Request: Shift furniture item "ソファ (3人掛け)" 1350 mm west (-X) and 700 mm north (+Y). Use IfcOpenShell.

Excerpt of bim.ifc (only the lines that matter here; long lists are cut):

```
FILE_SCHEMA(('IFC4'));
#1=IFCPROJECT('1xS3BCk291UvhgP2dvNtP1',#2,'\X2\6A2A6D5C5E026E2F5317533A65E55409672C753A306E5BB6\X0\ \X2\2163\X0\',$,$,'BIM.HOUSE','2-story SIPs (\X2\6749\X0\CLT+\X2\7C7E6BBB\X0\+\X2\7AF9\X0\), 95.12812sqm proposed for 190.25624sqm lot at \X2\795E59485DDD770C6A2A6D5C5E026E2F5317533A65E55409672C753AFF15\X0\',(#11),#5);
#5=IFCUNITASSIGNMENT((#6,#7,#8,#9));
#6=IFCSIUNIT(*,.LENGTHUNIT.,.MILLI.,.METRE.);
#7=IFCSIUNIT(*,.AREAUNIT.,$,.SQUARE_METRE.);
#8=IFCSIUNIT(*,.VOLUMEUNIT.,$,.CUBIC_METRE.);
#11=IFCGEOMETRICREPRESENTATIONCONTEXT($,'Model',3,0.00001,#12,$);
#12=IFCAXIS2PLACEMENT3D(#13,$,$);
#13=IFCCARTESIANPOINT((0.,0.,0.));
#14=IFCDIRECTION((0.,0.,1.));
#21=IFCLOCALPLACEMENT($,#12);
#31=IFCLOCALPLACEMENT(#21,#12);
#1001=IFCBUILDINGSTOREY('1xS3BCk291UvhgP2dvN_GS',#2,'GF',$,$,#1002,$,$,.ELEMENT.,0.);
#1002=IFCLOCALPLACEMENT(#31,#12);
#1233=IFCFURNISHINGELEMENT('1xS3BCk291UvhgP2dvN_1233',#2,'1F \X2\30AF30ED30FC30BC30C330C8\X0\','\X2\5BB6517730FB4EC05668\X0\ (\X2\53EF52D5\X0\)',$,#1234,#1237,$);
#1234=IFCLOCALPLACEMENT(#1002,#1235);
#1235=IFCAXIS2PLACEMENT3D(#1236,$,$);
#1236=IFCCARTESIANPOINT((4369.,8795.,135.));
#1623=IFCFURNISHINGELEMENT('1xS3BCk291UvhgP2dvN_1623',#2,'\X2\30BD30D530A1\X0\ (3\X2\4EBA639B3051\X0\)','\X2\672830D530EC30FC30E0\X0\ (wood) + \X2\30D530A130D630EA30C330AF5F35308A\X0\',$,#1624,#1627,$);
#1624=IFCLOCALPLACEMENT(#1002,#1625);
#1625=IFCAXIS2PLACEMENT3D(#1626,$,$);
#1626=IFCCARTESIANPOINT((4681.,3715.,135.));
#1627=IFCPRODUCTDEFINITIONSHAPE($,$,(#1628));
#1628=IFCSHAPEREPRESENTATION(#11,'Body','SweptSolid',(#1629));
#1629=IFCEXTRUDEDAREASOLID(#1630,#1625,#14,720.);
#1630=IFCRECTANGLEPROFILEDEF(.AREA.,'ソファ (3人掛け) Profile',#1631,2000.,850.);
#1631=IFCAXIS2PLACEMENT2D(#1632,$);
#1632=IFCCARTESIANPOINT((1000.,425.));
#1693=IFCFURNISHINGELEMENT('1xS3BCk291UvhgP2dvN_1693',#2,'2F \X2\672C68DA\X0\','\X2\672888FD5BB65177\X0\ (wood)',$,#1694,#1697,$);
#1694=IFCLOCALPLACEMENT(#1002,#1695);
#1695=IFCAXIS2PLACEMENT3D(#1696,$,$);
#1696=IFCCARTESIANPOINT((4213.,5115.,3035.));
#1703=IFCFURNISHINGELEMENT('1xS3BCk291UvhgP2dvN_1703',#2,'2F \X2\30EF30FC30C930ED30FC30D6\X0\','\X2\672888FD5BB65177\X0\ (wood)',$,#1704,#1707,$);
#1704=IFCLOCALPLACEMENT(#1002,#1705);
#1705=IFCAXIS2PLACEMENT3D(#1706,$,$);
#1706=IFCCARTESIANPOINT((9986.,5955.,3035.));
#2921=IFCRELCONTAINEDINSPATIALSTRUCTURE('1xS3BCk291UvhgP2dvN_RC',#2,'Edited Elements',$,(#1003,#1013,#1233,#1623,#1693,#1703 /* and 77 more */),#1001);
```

```python
import ifcopenshell
import ifcopenshell.api.geometry
import ifcopenshell.util.placement

model = ifcopenshell.open("bim.ifc")

item = model.by_guid("1xS3BCk291UvhgP2dvN_1623")
matrix = ifcopenshell.util.placement.get_local_placement(item.ObjectPlacement)
matrix[0, 3] -= 1350.0
matrix[1, 3] += 700.0
ifcopenshell.api.geometry.edit_object_placement(model, product=item, matrix=matrix, is_si=False)

print(ifcopenshell.util.placement.get_local_placement(item.ObjectPlacement).round(3) + 0.0)

model.write("bim_rev.ifc")
```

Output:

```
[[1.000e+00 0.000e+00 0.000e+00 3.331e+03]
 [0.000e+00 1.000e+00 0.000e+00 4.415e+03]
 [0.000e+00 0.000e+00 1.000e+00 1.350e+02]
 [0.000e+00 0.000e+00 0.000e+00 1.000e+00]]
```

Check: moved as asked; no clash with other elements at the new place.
